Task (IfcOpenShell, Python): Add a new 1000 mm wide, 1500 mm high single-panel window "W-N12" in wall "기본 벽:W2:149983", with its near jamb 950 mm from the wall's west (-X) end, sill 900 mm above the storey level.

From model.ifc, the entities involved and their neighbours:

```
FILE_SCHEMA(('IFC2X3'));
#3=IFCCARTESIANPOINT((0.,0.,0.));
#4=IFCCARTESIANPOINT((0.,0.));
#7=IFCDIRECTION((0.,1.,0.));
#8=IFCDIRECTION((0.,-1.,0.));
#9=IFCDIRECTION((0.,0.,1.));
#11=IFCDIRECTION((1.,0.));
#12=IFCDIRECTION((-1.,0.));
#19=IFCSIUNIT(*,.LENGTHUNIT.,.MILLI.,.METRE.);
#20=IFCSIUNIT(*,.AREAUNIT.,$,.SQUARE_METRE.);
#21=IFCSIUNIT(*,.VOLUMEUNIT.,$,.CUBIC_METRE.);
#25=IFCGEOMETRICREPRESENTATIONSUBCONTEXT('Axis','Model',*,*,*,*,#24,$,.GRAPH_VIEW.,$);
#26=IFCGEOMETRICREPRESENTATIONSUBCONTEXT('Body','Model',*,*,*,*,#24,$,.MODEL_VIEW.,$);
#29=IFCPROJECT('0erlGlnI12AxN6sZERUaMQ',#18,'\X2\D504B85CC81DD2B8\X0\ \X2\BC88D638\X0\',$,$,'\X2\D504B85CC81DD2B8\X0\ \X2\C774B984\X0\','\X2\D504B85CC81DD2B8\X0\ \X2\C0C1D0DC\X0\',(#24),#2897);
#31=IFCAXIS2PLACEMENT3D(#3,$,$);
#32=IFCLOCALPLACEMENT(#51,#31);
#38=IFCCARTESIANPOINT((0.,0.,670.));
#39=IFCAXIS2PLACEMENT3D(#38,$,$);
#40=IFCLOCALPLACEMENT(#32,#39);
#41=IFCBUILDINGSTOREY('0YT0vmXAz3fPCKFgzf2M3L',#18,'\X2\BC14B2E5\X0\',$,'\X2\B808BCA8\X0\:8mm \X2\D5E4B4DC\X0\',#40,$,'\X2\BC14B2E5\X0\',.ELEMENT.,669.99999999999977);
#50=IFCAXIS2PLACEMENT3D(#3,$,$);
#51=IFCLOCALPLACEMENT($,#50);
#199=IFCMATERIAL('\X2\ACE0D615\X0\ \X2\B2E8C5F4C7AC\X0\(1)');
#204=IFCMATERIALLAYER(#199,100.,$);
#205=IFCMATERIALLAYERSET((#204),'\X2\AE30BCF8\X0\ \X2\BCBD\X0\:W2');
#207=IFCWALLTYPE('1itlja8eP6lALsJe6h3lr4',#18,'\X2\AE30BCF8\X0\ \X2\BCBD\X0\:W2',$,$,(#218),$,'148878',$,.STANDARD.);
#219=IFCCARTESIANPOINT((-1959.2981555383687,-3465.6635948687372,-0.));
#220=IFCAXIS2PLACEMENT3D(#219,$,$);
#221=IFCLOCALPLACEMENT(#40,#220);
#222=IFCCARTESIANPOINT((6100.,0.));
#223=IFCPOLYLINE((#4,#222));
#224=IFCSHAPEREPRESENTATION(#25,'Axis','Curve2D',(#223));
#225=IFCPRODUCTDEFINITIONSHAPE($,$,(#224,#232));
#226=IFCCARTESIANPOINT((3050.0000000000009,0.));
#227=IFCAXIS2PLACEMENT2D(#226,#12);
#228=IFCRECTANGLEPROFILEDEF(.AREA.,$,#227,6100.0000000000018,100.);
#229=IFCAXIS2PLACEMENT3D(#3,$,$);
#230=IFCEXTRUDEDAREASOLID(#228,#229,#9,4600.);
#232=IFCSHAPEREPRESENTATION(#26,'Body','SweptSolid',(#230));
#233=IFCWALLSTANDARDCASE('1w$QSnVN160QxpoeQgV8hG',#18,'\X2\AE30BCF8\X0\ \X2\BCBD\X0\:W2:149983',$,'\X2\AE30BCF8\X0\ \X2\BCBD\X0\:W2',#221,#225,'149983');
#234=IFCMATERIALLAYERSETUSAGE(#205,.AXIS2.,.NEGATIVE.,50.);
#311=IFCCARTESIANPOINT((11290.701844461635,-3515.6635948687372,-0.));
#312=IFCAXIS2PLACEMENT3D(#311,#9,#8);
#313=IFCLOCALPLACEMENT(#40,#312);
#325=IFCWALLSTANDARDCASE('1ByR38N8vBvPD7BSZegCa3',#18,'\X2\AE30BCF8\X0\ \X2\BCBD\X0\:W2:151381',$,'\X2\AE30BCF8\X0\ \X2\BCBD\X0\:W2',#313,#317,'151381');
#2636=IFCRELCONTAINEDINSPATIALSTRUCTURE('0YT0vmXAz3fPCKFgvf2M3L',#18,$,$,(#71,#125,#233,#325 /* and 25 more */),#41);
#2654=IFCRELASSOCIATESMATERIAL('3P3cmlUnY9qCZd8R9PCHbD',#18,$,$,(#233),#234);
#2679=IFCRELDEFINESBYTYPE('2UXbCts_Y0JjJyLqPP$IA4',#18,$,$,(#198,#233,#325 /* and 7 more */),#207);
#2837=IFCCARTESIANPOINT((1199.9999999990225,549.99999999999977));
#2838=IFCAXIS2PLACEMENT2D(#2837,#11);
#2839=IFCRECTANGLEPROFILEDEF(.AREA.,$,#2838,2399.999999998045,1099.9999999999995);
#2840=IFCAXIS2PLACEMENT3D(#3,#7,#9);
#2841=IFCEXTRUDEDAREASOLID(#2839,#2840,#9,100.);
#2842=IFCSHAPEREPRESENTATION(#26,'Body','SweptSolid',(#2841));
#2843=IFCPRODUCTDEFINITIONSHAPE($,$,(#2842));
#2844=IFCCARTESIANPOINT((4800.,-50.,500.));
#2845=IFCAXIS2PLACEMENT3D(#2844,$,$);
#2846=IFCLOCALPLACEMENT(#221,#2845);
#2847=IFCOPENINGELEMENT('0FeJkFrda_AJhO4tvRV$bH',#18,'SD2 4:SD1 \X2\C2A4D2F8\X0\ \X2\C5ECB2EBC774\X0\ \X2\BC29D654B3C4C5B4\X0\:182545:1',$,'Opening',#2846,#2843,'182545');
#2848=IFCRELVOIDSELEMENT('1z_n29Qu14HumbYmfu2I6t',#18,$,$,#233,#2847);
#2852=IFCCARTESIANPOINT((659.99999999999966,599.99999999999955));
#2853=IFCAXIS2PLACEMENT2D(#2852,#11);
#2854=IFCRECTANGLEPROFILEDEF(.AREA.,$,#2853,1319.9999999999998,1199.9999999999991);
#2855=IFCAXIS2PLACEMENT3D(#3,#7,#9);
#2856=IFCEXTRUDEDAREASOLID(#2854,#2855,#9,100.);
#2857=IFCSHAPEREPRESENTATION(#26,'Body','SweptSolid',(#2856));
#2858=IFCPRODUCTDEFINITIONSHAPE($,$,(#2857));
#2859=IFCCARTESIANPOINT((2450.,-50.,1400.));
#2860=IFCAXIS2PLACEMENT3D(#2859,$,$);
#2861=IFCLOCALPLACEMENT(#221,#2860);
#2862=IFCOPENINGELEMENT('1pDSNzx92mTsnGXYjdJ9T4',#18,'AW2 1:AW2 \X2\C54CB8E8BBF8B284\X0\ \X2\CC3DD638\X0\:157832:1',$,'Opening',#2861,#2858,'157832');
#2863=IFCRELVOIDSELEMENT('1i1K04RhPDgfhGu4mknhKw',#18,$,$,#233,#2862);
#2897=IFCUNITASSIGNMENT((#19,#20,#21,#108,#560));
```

```python
import numpy as np
import ifcopenshell
import ifcopenshell.api.feature
import ifcopenshell.api.geometry
import ifcopenshell.api.root
import ifcopenshell.api.spatial
import ifcopenshell.api.type
import ifcopenshell.geom
import ifcopenshell.util.element
import ifcopenshell.util.placement
import ifcopenshell.util.representation
import ifcopenshell.util.shape
import ifcopenshell.util.unit

model = ifcopenshell.open("model.ifc")
unit_scale = ifcopenshell.util.unit.calculate_unit_scale(model)
settings = ifcopenshell.geom.settings()


def volume(element):
    """Net volume in cubic metres, openings subtracted."""
    shape = ifcopenshell.geom.create_shape(settings, element)
    return ifcopenshell.util.shape.get_volume(shape.geometry)


wall = model.by_guid("1w$QSnVN160QxpoeQgV8hG")
storey = ifcopenshell.util.element.get_container(wall, ifc_class="IfcBuildingStorey")
context = ifcopenshell.util.representation.get_context(model, "Model", "Body", "MODEL_VIEW")
before = volume(wall)

width, height, from_end, sill = 1, 1.5, 0.95, 0.9  # metres

# The wall runs along its own X axis, and the end named is its -X end.
wall_shape = ifcopenshell.geom.create_shape(settings, wall)
x, y, z = ifcopenshell.util.shape.get_vertices(wall_shape.geometry).T
start = x.min() + from_end
face, thickness = float(y.min()), float(y.max() - y.min())
wall_matrix = ifcopenshell.util.placement.get_local_placement(wall.ObjectPlacement)
level = ifcopenshell.util.placement.get_local_placement(storey.ObjectPlacement)[2, 3]


def in_wall(x, y):
    """Placement at x, y metres in the wall's axes, at sill height."""
    matrix = wall_matrix.copy()
    matrix[:, 3] = wall_matrix @ np.array([x / unit_scale, y / unit_scale, 0.0, 1.0])
    matrix[2, 3] = level + sill / unit_scale
    return matrix


# Opening: a box that overshoots both wall faces by 50 mm.
opening = ifcopenshell.api.root.create_entity(model, ifc_class="IfcOpeningElement")
box = ifcopenshell.api.geometry.add_wall_representation(
    model, context=context, length=width, height=height, thickness=thickness + 0.1
)
ifcopenshell.api.geometry.assign_representation(model, product=opening, representation=box)
ifcopenshell.api.geometry.edit_object_placement(model, product=opening, matrix=in_wall(start, face - 0.05), is_si=False)
ifcopenshell.api.feature.add_feature(model, feature=opening, element=wall)

window = ifcopenshell.api.root.create_entity(model, ifc_class="IfcWindow", name="W-N12")
window.OverallWidth, window.OverallHeight = width / unit_scale, height / unit_scale
body = ifcopenshell.api.geometry.add_window_representation(
    model,
    context=context,
    overall_width=window.OverallWidth,
    overall_height=window.OverallHeight,
    partition_type="SINGLE_PANEL",
)
ifcopenshell.api.geometry.assign_representation(model, product=window, representation=body)
ifcopenshell.api.spatial.assign_container(model, products=[window], relating_structure=storey)
fills = ifcopenshell.api.feature.add_filling(model, opening=opening, element=window)
fills.OwnerHistory = window.OwnerHistory  # required in IFC2X3

# IFC2X3 keeps the operation on the window style.
style = ifcopenshell.api.root.create_entity(model, ifc_class="IfcWindowStyle", name="W-N12")
style.OperationType, style.ConstructionType = "SINGLE_PANEL", "NOTDEFINED"
style.ParameterTakesPrecedence = style.Sizeable = False
ifcopenshell.api.type.assign_type(model, related_objects=[window], relating_type=style)

# Centre the window in the wall's thickness.
ifcopenshell.api.geometry.edit_object_placement(model, product=window, matrix=in_wall(start, face), is_si=False)
window_shape = ifcopenshell.geom.create_shape(settings, window)
depth = ifcopenshell.util.shape.get_vertices(window_shape.geometry)[:, 1]
offset = face + thickness / 2 - (depth.min() + depth.max()) / 2
ifcopenshell.api.geometry.edit_object_placement(model, product=window, matrix=in_wall(start, offset), is_si=False)

after = volume(wall)

print(f"wall volume {before:.3f} -> {after:.3f} m3")

model.write("model-out.ifc")
```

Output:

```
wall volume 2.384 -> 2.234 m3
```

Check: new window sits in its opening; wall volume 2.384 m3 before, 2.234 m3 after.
